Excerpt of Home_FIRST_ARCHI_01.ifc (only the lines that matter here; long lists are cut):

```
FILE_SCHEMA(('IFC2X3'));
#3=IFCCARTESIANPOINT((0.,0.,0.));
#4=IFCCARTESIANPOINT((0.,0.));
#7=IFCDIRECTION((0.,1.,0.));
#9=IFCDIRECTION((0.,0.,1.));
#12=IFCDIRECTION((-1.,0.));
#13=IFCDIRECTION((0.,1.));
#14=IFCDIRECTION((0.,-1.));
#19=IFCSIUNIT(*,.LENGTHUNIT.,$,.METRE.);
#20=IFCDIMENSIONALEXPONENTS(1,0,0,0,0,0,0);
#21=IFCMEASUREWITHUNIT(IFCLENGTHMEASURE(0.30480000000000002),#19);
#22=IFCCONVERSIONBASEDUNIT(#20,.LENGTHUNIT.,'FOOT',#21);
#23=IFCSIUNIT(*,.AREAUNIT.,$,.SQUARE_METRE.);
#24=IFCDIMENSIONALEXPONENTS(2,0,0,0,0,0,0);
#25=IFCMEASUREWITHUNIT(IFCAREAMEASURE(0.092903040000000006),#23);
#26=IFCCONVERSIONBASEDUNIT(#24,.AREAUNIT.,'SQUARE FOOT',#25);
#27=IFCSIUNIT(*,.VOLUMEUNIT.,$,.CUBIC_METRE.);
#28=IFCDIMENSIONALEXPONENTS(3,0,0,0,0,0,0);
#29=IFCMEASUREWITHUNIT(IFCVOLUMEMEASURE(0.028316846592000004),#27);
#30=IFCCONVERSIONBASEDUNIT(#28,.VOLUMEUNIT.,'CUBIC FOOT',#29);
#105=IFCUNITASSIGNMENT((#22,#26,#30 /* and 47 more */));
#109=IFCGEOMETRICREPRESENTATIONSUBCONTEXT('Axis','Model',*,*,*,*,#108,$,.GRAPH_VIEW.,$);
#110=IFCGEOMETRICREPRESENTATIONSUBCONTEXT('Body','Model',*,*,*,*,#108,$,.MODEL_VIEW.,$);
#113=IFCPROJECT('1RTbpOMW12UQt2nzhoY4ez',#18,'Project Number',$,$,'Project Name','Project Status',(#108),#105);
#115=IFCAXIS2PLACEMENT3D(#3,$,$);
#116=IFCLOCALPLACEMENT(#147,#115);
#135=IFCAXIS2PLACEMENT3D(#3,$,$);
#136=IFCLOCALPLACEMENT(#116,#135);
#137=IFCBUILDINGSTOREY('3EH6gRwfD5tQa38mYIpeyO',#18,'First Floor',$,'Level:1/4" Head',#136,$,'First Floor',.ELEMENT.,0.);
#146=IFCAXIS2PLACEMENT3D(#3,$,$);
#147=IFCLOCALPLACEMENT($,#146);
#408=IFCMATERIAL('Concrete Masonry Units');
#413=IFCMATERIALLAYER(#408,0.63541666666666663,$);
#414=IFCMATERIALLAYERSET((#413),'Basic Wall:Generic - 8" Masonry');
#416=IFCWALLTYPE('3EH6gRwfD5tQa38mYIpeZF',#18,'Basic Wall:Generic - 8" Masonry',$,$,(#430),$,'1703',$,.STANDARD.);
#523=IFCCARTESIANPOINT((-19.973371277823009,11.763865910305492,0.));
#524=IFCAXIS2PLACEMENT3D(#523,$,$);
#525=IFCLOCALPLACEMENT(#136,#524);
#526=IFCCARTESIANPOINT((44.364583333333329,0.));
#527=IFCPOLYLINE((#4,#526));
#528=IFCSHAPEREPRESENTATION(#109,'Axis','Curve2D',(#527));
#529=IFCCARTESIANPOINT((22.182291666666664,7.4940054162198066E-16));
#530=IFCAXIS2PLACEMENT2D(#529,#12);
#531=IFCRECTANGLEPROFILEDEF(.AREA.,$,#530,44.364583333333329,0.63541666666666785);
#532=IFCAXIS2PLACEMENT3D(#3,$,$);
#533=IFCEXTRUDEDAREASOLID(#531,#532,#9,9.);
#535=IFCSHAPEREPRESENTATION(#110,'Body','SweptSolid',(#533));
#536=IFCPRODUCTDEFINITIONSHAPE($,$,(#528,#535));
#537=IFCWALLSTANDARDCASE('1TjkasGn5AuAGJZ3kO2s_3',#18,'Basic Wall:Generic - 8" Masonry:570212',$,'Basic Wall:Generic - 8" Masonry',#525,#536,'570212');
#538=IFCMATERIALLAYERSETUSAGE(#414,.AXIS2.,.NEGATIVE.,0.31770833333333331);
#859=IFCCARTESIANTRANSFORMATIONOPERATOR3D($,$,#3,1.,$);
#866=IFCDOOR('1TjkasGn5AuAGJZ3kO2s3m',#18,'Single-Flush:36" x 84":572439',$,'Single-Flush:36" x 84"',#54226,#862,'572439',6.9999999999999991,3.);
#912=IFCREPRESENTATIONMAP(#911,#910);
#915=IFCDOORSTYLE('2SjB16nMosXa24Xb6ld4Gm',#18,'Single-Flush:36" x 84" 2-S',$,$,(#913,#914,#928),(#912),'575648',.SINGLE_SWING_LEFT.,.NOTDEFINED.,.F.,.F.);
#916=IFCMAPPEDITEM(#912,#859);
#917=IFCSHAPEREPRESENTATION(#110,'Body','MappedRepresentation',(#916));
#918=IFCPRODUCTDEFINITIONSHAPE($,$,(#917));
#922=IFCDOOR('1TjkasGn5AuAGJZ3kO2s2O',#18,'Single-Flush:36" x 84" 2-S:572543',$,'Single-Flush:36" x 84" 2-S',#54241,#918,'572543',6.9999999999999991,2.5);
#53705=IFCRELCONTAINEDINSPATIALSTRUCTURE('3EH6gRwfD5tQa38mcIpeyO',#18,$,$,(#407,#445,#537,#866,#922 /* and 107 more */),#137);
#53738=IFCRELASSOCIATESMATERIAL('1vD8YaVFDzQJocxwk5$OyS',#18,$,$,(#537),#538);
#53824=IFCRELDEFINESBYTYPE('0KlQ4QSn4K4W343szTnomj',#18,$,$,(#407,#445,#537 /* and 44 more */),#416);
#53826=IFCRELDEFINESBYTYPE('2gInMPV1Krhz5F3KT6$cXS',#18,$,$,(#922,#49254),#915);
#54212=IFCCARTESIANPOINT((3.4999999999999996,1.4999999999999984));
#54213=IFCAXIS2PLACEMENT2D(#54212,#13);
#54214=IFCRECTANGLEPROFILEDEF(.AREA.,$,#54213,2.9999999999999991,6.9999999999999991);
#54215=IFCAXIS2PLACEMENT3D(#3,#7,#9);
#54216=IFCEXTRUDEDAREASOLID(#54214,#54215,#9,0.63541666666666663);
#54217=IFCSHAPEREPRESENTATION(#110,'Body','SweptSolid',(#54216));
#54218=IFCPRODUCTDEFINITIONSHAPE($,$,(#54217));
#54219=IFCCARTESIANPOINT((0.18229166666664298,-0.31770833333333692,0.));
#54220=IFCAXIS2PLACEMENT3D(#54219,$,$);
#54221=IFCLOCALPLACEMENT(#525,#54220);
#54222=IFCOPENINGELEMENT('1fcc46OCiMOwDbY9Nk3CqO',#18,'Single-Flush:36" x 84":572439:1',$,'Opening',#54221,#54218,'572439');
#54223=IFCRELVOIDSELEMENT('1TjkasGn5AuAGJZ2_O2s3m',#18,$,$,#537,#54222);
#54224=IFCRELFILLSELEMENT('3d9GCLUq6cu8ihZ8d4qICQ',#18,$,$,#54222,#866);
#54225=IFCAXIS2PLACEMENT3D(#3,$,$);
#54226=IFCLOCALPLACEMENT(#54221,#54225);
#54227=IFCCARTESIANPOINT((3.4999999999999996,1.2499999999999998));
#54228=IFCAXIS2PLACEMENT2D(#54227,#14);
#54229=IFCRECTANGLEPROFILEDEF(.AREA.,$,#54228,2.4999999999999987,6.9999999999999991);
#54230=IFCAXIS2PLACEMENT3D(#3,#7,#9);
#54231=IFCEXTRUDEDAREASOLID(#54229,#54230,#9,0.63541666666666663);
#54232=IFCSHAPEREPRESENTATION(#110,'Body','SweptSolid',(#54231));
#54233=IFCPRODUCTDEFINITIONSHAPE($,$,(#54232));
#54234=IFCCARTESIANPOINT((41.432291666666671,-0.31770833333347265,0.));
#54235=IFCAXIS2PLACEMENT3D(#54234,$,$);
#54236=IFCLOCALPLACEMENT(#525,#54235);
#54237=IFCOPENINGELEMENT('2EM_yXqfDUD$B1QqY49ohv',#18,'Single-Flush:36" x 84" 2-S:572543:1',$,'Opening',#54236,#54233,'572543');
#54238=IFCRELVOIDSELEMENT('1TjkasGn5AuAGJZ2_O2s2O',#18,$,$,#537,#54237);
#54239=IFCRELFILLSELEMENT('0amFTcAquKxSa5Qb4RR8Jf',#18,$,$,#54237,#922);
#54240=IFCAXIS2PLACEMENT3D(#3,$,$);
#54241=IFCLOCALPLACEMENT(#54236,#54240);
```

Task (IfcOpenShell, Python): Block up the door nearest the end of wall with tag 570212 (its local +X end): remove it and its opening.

```python
import ifcopenshell
import ifcopenshell.api.feature
import ifcopenshell.api.root
import ifcopenshell.geom
import ifcopenshell.util.shape

model = ifcopenshell.open("Home_FIRST_ARCHI_01.ifc")
settings = ifcopenshell.geom.settings()


def volume(element):
    """Net volume in cubic metres, openings subtracted."""
    shape = ifcopenshell.geom.create_shape(settings, element)
    return ifcopenshell.util.shape.get_volume(shape.geometry)


door = model.by_guid("1TjkasGn5AuAGJZ3kO2s2O")
opening = door.FillsVoids[0].RelatingOpeningElement
wall = opening.VoidsElements[0].RelatingBuildingElement
before = volume(wall)

ifcopenshell.api.root.remove_product(model, product=door)
ifcopenshell.api.feature.remove_feature(model, feature=opening)

after = volume(wall)

print(f"wall volume {before:.3f} -> {after:.3f} m3")

model.write("Home_FIRST_ARCHI_01_rev.ifc")
```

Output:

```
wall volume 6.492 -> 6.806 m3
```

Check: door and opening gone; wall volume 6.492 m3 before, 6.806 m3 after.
